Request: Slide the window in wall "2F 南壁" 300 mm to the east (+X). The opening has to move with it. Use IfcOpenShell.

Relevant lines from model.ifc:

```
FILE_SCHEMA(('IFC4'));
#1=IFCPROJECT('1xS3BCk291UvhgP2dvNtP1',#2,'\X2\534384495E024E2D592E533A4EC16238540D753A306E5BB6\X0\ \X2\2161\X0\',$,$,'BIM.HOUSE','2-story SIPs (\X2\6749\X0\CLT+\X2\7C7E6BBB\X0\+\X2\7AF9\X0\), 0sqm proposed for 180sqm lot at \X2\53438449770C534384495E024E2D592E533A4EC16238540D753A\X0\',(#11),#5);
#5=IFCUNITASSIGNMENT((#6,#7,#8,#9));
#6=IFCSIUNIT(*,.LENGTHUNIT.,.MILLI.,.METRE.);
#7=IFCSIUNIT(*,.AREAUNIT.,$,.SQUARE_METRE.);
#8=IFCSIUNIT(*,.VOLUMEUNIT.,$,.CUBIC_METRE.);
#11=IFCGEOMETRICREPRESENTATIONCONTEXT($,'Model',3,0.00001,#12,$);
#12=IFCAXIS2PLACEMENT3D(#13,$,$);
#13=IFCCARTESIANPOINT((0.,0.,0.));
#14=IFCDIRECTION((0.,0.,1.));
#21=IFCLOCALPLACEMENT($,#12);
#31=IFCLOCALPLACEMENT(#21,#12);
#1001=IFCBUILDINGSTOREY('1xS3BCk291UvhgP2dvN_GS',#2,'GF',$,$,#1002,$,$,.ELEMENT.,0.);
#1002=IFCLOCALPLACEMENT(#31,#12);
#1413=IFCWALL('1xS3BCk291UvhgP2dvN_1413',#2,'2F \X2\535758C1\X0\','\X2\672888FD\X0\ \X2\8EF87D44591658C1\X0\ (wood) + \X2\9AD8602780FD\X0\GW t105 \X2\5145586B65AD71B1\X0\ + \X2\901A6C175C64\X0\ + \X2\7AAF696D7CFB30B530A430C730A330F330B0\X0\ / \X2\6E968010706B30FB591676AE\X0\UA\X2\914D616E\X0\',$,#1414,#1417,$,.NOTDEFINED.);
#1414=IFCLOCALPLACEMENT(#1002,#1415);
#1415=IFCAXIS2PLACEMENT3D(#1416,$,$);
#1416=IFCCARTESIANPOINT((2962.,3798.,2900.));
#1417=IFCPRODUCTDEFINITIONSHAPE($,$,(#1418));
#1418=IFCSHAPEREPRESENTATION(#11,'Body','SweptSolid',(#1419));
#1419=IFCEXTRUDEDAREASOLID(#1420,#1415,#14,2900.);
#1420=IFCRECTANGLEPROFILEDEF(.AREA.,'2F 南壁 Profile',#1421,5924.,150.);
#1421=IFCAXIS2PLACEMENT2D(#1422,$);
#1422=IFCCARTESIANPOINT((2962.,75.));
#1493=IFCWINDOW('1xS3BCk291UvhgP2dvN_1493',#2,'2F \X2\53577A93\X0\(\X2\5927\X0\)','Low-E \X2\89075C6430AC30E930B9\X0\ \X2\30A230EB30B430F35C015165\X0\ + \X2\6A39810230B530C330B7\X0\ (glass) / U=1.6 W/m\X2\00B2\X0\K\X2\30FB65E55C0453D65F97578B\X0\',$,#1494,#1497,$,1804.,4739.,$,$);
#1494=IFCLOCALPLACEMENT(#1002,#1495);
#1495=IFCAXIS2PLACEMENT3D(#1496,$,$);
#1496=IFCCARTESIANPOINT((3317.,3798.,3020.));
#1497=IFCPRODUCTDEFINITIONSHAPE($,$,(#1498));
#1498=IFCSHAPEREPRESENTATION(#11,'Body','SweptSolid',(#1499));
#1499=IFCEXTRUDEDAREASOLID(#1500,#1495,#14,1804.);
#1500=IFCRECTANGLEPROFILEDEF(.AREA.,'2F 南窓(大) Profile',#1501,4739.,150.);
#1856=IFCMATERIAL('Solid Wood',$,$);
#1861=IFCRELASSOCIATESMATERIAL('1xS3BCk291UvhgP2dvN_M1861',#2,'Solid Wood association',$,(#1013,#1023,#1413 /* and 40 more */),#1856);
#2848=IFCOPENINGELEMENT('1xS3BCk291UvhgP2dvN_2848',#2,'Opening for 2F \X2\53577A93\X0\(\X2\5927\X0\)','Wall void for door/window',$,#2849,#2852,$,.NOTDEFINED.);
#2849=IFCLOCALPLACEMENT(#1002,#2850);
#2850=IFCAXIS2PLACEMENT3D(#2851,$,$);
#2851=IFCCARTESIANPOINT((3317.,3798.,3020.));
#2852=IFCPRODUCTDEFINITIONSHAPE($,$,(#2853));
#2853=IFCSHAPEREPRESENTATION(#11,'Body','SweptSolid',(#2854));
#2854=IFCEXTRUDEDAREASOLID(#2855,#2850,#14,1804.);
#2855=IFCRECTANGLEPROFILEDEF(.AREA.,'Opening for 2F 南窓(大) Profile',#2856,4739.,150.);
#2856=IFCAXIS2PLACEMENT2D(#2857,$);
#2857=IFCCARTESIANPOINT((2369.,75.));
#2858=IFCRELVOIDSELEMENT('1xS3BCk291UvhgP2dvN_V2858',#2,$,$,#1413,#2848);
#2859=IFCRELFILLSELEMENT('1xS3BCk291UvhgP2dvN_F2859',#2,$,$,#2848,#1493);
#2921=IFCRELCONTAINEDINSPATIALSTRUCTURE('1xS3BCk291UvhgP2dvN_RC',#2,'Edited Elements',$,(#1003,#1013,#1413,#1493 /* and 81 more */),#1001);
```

```python
import ifcopenshell
import ifcopenshell.api.geometry
import ifcopenshell.util.placement
import ifcopenshell.util.unit

model = ifcopenshell.open("model.ifc")
unit_scale = ifcopenshell.util.unit.calculate_unit_scale(model)

window = model.by_id(1493)
opening = window.FillsVoids[0].RelatingOpeningElement
wall = opening.VoidsElements[0].RelatingBuildingElement

wall_matrix = ifcopenshell.util.placement.get_local_placement(wall.ObjectPlacement)
shift = wall_matrix[:3, 0] * 0.3 / unit_scale
before = ifcopenshell.util.placement.get_local_placement(window.ObjectPlacement)[:3, 3].copy()

# The window is not placed relative to its opening, so move both.
for product in (opening, window):
    matrix = ifcopenshell.util.placement.get_local_placement(product.ObjectPlacement)
    matrix[:3, 3] += shift
    ifcopenshell.api.geometry.edit_object_placement(model, product=product, matrix=matrix, is_si=False)

after = ifcopenshell.util.placement.get_local_placement(window.ObjectPlacement)[:3, 3]
print("window moved by", (after - before).round(3) + 0.0)

model.write("model_updated.ifc")
```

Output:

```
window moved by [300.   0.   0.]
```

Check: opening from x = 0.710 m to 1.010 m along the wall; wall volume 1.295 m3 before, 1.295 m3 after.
